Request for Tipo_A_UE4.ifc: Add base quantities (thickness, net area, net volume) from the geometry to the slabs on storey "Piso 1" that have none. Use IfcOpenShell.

First a look at what the model holds.

```python
import ifcopenshell
import ifcopenshell.util.element
import ifcopenshell.util.unit

model = ifcopenshell.open("Tipo_A_UE4.ifc")
print(model.schema)
for unit_type in ("LENGTHUNIT", "AREAUNIT", "VOLUMEUNIT"):
    print(unit_type, ifcopenshell.util.unit.calculate_unit_scale(model, unit_type))
storey = next(s for s in model.by_type("IfcBuildingStorey") if s.Name == "Piso 1")
slabs = [e for e in ifcopenshell.util.element.get_decomposition(storey) if e.is_a("IfcSlab")]
for e in sorted(slabs, key=lambda e: e.id()):
    print(e.id(), e.is_a(), e.Name, list(ifcopenshell.util.element.get_psets(e, qtos_only=True)), sep=" | ")
```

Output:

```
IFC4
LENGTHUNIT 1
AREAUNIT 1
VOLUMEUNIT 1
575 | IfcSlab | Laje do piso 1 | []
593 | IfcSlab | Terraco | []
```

```python
import ifcopenshell
import ifcopenshell.api.pset
import ifcopenshell.geom
import ifcopenshell.util.element
import ifcopenshell.util.shape
import ifcopenshell.util.unit

model = ifcopenshell.open("Tipo_A_UE4.ifc")
unit_scale = ifcopenshell.util.unit.calculate_unit_scale(model)
area_scale = ifcopenshell.util.unit.calculate_unit_scale(model, "AREAUNIT")
volume_scale = ifcopenshell.util.unit.calculate_unit_scale(model, "VOLUMEUNIT")
settings = ifcopenshell.geom.settings()

storey = next(s for s in model.by_type("IfcBuildingStorey") if s.Name == "Piso 1")
slabs = [e for e in ifcopenshell.util.element.get_decomposition(storey) if e.is_a("IfcSlab")]

for e in sorted(slabs, key=lambda e: e.id()):
    if ifcopenshell.util.element.get_psets(e, qtos_only=True, should_inherit=False):
        continue
    # Geometry comes back in metres, in the element's own axes.
    shape = ifcopenshell.geom.create_shape(settings, e)
    values = {
        "Width": ifcopenshell.util.shape.get_z(shape.geometry) / unit_scale,
        "NetArea": ifcopenshell.util.shape.get_footprint_area(shape.geometry) / area_scale,
        "NetVolume": ifcopenshell.util.shape.get_volume(shape.geometry) / volume_scale,
    }
    qto = ifcopenshell.api.pset.add_qto(model, product=e, name="Qto_SlabBaseQuantities")
    ifcopenshell.api.pset.edit_qto(model, qto=qto, properties=values)
    print(e.id(), {k: round(v, 3) for k, v in values.items()})

model.write("Tipo_A_UE4_v2.ifc")
```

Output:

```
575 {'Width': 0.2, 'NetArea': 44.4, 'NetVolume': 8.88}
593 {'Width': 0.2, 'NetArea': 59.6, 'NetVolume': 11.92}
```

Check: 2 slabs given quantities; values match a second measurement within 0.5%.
